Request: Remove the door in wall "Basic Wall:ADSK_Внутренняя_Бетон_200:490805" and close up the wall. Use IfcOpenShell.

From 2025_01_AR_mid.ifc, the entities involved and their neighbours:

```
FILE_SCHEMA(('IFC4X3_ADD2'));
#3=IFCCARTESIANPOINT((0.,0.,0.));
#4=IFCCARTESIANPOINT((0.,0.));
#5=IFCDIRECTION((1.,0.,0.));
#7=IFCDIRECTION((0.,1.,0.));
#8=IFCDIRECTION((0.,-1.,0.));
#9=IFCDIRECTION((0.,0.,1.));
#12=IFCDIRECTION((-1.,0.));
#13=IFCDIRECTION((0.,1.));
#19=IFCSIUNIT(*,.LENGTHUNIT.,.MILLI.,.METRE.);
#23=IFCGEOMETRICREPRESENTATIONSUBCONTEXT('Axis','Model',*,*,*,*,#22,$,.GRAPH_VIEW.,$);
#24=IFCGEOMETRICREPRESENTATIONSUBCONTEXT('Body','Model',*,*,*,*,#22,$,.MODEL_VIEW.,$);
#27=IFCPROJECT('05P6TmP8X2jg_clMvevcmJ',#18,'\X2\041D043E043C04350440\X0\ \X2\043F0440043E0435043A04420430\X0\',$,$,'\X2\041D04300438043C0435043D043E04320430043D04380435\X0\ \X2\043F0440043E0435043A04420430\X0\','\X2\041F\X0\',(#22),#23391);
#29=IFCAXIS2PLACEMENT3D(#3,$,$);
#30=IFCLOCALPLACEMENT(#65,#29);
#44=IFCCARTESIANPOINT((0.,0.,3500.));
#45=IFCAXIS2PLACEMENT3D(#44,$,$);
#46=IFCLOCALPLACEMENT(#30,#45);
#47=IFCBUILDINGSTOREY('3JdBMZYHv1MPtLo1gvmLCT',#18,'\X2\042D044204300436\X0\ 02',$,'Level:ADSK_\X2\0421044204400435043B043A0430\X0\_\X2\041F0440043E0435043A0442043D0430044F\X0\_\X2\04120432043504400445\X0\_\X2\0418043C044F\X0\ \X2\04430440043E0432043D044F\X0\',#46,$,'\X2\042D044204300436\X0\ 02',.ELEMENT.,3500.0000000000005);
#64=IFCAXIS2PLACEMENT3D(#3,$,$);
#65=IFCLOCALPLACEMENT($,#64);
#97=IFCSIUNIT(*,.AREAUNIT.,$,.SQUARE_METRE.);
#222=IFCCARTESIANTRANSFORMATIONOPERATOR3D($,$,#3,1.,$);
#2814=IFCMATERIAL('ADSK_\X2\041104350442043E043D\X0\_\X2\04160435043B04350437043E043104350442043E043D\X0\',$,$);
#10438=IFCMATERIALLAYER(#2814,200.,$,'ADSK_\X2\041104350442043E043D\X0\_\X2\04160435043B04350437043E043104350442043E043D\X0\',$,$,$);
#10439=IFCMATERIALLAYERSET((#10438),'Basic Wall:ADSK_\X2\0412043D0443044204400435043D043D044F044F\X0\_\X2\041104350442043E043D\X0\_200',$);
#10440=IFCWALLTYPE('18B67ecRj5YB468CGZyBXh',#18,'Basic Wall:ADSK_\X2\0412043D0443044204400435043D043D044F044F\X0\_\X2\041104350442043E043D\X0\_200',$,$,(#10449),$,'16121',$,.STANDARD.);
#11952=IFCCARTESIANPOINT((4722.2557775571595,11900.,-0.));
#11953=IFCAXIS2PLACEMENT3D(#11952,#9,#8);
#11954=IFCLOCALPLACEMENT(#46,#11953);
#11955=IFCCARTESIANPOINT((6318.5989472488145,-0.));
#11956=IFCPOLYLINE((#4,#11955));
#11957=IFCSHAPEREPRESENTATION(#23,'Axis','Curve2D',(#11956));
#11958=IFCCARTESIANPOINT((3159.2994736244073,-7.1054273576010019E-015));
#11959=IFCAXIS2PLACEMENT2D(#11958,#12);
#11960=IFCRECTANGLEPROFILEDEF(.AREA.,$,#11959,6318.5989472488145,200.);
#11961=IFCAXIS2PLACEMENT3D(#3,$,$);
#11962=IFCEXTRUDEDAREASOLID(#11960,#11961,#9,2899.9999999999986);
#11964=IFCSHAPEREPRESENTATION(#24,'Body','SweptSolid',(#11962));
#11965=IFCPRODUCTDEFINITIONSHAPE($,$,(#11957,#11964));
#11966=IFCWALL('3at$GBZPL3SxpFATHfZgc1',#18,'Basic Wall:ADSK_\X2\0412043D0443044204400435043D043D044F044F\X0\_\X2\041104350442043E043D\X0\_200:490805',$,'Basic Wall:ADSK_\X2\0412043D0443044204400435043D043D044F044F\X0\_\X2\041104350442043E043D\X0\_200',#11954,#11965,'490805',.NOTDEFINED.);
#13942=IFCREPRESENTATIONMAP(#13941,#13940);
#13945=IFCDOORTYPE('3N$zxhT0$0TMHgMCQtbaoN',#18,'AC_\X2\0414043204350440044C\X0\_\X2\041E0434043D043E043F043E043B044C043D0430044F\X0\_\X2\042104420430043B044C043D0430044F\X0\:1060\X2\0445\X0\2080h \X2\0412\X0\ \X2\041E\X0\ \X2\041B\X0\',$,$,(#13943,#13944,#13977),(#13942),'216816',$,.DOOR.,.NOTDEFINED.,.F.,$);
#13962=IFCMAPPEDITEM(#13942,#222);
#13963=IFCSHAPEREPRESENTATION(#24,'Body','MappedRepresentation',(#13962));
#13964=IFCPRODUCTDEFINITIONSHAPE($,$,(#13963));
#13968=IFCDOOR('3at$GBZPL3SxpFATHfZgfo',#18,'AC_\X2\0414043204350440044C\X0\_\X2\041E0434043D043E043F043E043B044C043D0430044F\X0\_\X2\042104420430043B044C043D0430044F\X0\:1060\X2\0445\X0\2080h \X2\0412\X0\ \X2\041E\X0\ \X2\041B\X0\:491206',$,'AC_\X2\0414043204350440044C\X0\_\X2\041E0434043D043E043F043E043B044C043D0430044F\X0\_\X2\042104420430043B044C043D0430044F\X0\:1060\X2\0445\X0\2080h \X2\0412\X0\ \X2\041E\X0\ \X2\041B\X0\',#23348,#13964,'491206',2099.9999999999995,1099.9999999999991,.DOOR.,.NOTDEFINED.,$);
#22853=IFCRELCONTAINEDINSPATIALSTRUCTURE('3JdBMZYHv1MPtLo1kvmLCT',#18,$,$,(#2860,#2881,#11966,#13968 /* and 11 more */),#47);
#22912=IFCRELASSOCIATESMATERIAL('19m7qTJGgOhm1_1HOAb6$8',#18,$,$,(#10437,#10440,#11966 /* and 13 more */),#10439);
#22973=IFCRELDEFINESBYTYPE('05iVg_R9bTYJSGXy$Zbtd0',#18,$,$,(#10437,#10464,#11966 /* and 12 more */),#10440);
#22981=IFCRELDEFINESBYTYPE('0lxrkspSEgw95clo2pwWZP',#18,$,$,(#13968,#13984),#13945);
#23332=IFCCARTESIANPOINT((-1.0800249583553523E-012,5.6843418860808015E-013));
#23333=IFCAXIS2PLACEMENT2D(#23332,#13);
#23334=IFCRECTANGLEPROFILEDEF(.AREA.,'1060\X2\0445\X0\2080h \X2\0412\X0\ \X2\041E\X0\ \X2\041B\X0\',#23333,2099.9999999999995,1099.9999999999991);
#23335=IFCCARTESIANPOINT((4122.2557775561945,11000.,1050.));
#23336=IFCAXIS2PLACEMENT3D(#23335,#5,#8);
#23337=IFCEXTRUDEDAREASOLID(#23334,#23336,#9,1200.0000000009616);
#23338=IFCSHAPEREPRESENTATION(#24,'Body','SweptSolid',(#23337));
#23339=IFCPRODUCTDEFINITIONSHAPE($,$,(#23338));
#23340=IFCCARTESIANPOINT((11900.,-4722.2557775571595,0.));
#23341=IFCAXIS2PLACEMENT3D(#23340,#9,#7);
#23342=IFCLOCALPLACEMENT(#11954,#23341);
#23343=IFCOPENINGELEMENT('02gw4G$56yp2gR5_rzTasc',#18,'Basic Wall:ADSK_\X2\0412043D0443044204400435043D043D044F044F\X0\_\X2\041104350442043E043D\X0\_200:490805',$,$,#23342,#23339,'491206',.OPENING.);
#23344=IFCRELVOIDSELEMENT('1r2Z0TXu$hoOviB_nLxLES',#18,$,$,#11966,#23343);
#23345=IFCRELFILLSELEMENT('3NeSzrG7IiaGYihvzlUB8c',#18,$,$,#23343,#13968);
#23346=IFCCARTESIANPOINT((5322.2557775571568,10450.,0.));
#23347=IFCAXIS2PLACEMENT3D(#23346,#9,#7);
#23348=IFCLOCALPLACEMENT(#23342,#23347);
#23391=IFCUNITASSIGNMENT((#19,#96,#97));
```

```python
import ifcopenshell
import ifcopenshell.api.feature
import ifcopenshell.api.root
import ifcopenshell.geom
import ifcopenshell.util.shape

model = ifcopenshell.open("2025_01_AR_mid.ifc")
settings = ifcopenshell.geom.settings()


def volume(element):
    """Net volume in cubic metres, openings subtracted."""
    shape = ifcopenshell.geom.create_shape(settings, element)
    return ifcopenshell.util.shape.get_volume(shape.geometry)


door = model.by_guid("3at$GBZPL3SxpFATHfZgfo")
opening = door.FillsVoids[0].RelatingOpeningElement
wall = opening.VoidsElements[0].RelatingBuildingElement
before = volume(wall)

ifcopenshell.api.root.remove_product(model, product=door)
ifcopenshell.api.feature.remove_feature(model, feature=opening)

after = volume(wall)

print(f"wall volume {before:.3f} -> {after:.3f} m3")

model.write("2025_01_AR_mid-out.ifc")
```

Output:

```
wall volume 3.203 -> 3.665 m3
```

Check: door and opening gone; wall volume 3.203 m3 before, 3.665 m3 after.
